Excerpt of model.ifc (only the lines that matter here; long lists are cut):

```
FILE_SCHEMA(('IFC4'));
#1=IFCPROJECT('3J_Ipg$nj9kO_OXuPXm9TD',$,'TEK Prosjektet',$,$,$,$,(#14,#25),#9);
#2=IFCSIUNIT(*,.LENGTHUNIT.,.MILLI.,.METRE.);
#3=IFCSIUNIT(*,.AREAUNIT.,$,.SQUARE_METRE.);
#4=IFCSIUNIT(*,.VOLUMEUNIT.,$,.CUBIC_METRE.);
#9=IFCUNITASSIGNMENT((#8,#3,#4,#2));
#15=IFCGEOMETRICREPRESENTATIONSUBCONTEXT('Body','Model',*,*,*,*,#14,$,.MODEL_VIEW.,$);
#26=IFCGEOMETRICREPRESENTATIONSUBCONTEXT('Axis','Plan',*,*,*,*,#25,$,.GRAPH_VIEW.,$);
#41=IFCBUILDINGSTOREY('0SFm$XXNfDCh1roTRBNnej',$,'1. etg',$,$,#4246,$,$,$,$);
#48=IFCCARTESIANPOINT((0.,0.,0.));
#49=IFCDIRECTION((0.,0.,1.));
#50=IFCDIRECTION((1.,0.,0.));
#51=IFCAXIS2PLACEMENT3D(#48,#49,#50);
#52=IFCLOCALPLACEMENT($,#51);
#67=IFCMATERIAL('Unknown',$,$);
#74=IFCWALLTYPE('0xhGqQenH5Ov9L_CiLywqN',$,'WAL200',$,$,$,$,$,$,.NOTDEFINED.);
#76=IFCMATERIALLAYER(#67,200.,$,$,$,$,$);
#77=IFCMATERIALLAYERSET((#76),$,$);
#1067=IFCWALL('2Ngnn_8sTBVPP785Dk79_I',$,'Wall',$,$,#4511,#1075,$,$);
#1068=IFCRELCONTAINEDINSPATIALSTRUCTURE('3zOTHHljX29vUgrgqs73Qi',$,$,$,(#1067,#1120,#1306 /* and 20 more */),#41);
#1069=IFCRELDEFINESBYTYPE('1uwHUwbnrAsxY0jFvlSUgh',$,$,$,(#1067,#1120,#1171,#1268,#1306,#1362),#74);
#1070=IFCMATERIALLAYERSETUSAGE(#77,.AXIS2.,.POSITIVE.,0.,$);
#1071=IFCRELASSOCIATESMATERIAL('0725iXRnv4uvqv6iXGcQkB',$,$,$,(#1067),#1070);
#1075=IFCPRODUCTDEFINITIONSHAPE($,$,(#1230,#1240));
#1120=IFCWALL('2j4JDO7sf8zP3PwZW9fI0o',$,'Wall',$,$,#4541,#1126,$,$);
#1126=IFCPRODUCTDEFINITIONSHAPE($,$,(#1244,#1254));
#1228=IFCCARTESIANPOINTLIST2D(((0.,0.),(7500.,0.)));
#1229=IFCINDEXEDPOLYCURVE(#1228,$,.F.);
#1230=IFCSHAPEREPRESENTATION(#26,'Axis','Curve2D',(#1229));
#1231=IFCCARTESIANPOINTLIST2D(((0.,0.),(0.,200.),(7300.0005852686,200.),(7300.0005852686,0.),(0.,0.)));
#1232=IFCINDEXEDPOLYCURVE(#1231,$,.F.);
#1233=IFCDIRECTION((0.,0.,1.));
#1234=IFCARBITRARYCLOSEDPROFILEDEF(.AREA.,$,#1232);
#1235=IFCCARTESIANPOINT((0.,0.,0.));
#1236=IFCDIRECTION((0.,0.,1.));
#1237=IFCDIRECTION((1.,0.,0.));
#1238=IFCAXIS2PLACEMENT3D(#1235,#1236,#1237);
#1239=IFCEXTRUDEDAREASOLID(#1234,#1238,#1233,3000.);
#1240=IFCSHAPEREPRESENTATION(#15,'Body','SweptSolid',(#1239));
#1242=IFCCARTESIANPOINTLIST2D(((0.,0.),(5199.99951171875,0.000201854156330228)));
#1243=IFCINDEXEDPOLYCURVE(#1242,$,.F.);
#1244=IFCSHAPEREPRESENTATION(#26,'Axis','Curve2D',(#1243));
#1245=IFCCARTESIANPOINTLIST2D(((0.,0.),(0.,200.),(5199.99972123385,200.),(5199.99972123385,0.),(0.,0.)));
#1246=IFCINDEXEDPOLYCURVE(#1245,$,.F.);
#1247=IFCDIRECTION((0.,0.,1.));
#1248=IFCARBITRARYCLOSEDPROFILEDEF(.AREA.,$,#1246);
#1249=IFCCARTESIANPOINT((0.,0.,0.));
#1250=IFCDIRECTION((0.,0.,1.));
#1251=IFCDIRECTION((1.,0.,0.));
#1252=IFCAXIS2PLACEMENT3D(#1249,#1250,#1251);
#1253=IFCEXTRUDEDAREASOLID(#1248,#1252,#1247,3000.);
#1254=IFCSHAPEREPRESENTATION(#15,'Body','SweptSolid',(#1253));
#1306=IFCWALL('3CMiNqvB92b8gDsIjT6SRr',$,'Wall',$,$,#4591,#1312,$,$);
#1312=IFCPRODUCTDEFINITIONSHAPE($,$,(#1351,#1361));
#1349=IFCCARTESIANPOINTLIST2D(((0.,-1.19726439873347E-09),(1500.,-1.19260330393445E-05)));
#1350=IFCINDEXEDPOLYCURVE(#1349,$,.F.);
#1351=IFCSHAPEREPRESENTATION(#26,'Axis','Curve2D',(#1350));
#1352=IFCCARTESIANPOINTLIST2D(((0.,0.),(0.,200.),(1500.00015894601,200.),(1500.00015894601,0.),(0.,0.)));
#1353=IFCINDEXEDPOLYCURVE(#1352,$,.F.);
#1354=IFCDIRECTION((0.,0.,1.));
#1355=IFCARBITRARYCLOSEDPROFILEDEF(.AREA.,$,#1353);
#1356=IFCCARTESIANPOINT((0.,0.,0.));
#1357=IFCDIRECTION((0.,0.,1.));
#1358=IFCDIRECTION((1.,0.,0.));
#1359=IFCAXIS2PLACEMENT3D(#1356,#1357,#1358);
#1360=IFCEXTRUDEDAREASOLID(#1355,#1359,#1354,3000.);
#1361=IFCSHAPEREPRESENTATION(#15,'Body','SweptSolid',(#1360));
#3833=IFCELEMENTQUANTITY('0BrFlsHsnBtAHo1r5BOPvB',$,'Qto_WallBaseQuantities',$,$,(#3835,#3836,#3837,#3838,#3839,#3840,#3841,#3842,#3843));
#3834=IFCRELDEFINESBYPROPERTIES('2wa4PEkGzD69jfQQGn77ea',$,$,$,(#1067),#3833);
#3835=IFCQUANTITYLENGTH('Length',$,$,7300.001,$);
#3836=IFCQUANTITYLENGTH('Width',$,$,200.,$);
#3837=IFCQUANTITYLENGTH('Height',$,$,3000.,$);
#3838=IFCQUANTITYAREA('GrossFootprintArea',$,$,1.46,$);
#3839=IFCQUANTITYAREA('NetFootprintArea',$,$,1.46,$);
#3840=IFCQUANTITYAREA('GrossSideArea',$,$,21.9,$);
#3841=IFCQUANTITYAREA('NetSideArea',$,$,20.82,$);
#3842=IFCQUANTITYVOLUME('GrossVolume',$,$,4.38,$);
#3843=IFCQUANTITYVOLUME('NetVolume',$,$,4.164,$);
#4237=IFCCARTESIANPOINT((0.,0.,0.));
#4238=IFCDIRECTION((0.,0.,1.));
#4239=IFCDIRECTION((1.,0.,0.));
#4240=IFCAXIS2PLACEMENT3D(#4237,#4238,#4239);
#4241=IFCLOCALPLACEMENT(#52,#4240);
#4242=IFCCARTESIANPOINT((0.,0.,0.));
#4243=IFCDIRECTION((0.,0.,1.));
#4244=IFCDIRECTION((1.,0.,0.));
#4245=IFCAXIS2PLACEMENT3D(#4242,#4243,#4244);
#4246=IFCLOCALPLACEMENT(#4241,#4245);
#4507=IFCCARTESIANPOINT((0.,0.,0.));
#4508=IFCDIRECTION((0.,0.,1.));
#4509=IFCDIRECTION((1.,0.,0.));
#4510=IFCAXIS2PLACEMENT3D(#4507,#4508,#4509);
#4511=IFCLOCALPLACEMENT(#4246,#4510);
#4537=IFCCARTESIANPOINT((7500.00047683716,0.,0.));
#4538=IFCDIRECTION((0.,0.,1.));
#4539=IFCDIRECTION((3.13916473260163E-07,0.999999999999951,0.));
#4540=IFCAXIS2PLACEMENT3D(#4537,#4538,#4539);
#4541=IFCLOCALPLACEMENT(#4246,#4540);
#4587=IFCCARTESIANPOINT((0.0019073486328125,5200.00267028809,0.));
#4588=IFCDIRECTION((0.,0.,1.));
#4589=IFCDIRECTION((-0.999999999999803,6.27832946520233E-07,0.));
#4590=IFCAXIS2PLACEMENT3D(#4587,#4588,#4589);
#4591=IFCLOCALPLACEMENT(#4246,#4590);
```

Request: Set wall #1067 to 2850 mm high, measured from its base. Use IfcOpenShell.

```python
import ifcopenshell
import ifcopenshell.api.pset
import ifcopenshell.geom
import ifcopenshell.util.element
import ifcopenshell.util.representation
import ifcopenshell.util.shape
import ifcopenshell.util.unit

model = ifcopenshell.open("model.ifc")
unit_scale = ifcopenshell.util.unit.calculate_unit_scale(model)
area_scale = ifcopenshell.util.unit.calculate_unit_scale(model, "AREAUNIT")
volume_scale = ifcopenshell.util.unit.calculate_unit_scale(model, "VOLUMEUNIT")
settings = ifcopenshell.geom.settings()


def volume(element):
    """Net volume in cubic metres, openings subtracted."""
    shape = ifcopenshell.geom.create_shape(settings, element)
    return ifcopenshell.util.shape.get_volume(shape.geometry)


wall = model.by_id(1067)
before = volume(wall)

body = ifcopenshell.util.representation.get_representation(wall, "Model", "Body")
solid = body.Items[0]
old_height = solid.Depth
solid.Depth = 2.85 / unit_scale
after = volume(wall)
thickness = 0.2  # wall thickness in metres

# Update the stored height, areas and volumes.
qto = model.by_id(ifcopenshell.util.element.get_pset(wall, "Qto_WallBaseQuantities", should_inherit=False)["id"])
ifcopenshell.api.pset.edit_qto(model, qto=qto, properties={
    "Height": solid.Depth,
    "GrossSideArea": ifcopenshell.util.element.get_pset(wall, "Qto_WallBaseQuantities", "GrossSideArea") * solid.Depth / old_height,
    "NetSideArea": after / thickness / area_scale,
    "GrossVolume": ifcopenshell.util.element.get_pset(wall, "Qto_WallBaseQuantities", "GrossVolume") * solid.Depth / old_height,
    "NetVolume": after / volume_scale,
})

print(f"height {old_height:g} -> {solid.Depth:g}, volume {before:.3f} -> {after:.3f} m3")

model.write("model-out.ifc")
```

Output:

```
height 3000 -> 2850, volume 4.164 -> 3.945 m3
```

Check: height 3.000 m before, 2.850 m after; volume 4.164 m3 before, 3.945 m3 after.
